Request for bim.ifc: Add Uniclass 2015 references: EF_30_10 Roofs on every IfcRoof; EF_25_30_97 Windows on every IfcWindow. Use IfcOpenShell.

First a look at what the model holds.

```python
import ifcopenshell

model = ifcopenshell.open("bim.ifc")
print(model.schema)
print("classifications:", [c.Name for c in model.by_type("IfcClassification")])
for ifc_class in ("IfcDoor", "IfcRoof", "IfcStair", "IfcWall", "IfcWindow"):
    print(ifc_class, len(model.by_type(ifc_class)))
```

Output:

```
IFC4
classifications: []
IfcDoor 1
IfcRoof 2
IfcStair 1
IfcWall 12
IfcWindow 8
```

```python
import ifcopenshell
import ifcopenshell.api.classification

model = ifcopenshell.open("bim.ifc")

system = ifcopenshell.api.classification.add_classification(model, classification="Uniclass 2015")

codes = {
    "IfcRoof": ("EF_30_10", "Roofs"),
    "IfcWindow": ("EF_25_30_97", "Windows"),
}
for ifc_class, (code, name) in codes.items():
    products = model.by_type(ifc_class)
    ifcopenshell.api.classification.add_reference(
        model, products=products, classification=system, identification=code, name=name
    )
    print(code, len(products))

model.write("bim_rev.ifc")
```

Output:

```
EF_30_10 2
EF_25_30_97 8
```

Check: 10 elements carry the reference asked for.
